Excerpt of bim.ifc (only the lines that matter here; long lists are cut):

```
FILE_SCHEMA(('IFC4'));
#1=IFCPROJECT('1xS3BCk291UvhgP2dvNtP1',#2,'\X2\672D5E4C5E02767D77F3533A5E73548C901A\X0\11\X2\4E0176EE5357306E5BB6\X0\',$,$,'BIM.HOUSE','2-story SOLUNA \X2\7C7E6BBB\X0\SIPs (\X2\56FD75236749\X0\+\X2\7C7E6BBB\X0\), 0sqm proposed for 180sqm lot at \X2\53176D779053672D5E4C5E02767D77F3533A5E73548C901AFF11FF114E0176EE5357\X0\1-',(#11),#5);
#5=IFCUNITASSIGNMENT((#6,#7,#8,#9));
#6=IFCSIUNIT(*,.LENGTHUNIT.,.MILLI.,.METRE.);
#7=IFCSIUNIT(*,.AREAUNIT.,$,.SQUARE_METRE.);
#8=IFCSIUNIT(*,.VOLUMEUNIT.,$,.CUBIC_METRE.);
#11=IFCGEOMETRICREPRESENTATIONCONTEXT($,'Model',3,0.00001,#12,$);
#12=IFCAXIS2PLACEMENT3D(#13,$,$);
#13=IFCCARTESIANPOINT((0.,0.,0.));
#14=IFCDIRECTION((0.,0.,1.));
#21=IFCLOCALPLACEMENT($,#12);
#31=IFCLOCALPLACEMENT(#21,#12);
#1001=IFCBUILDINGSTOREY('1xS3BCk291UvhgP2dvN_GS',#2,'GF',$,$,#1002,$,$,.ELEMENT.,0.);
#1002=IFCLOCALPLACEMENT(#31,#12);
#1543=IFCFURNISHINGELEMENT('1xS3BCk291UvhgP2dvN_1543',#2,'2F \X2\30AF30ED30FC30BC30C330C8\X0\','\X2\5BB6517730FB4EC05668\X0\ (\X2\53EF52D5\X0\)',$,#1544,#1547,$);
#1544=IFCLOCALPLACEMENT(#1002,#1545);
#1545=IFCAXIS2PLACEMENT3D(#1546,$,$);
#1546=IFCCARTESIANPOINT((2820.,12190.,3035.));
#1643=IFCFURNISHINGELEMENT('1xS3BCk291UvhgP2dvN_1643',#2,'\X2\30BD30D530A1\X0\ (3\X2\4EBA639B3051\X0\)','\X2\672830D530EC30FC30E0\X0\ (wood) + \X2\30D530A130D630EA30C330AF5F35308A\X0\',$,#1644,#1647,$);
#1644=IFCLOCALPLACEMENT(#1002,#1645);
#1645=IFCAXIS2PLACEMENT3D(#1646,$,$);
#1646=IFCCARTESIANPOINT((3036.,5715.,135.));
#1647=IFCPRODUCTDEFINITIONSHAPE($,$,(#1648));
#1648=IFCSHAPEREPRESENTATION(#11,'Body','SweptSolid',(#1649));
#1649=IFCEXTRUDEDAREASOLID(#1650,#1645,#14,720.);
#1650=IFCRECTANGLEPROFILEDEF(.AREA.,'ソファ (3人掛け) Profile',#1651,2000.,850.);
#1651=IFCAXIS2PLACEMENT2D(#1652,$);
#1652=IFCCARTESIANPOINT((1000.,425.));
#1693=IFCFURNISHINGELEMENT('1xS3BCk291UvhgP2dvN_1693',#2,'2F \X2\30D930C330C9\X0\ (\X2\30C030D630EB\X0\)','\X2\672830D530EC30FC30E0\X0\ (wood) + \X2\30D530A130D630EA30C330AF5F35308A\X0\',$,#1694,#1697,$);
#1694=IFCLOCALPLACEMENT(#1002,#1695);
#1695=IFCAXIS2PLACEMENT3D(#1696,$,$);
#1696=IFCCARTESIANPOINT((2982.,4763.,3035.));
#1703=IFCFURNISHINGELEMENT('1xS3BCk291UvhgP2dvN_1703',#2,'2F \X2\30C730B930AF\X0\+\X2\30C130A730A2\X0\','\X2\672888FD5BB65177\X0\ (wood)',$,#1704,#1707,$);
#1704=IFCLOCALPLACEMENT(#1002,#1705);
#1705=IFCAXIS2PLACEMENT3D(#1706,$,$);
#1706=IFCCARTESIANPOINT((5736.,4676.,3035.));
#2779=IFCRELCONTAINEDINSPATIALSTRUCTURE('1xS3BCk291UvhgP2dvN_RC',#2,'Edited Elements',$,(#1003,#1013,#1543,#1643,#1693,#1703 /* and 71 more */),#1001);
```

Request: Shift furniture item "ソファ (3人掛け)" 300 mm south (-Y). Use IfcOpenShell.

```python
import ifcopenshell
import ifcopenshell.api.geometry
import ifcopenshell.util.placement

model = ifcopenshell.open("bim.ifc")

item = model.by_guid("1xS3BCk291UvhgP2dvN_1643")
matrix = ifcopenshell.util.placement.get_local_placement(item.ObjectPlacement)
matrix[1, 3] -= 300.0
ifcopenshell.api.geometry.edit_object_placement(model, product=item, matrix=matrix, is_si=False)

print(ifcopenshell.util.placement.get_local_placement(item.ObjectPlacement).round(3) + 0.0)

model.write("bim_updated.ifc")
```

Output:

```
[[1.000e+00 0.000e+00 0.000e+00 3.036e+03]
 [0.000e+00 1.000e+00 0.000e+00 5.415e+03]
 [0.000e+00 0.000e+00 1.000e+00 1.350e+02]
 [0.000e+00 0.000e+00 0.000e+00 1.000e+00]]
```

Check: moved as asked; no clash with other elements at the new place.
